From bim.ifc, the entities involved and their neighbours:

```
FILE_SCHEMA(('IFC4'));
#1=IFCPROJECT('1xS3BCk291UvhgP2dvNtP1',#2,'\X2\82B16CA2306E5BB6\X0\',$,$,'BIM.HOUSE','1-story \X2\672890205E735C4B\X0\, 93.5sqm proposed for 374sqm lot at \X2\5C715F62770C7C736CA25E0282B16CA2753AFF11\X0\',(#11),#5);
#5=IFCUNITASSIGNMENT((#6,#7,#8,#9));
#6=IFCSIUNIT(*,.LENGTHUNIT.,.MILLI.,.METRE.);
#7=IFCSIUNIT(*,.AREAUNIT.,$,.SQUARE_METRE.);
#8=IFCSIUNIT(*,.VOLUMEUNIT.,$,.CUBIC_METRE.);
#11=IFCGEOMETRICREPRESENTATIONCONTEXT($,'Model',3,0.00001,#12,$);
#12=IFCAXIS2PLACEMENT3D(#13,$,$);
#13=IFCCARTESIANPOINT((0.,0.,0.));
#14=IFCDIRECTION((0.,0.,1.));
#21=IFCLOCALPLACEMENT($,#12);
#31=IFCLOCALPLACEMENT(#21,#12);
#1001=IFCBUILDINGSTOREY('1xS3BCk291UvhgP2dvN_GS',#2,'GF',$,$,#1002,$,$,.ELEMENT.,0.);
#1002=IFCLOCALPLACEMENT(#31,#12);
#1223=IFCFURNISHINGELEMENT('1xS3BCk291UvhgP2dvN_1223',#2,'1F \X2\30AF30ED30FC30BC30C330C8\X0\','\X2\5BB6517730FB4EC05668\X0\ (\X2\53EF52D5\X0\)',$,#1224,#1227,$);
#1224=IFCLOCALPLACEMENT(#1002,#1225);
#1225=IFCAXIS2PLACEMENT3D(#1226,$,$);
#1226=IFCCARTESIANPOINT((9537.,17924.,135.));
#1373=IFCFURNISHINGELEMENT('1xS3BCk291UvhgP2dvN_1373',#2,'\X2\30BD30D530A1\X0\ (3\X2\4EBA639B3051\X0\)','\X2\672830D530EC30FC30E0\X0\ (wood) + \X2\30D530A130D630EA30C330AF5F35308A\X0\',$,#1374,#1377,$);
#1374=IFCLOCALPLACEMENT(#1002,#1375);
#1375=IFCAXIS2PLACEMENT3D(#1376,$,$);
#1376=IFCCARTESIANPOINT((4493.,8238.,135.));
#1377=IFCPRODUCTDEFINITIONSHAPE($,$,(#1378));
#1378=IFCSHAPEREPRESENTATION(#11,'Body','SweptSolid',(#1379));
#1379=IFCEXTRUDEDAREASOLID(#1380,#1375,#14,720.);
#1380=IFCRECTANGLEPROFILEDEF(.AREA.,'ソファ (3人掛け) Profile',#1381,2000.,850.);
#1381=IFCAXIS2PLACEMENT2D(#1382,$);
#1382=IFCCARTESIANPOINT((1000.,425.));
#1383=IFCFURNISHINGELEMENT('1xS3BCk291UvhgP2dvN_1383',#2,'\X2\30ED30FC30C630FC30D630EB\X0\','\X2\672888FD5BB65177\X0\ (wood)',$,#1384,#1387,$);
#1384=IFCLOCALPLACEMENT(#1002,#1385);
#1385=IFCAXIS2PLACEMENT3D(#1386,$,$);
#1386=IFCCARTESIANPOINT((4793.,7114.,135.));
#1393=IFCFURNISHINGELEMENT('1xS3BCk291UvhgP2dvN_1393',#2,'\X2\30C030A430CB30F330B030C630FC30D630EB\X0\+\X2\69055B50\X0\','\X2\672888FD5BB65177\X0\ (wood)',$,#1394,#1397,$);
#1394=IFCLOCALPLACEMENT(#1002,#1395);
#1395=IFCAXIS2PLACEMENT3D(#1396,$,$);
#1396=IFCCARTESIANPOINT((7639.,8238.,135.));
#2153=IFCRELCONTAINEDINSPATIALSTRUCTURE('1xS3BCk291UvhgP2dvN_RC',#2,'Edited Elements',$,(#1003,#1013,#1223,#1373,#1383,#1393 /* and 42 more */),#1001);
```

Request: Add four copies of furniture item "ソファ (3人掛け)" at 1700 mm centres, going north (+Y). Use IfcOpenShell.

```python
import numpy as np
import ifcopenshell
import ifcopenshell.api.geometry
import ifcopenshell.api.root
import ifcopenshell.util.element
import ifcopenshell.util.placement
import ifcopenshell.util.unit

model = ifcopenshell.open("bim.ifc")
unit_scale = ifcopenshell.util.unit.calculate_unit_scale(model)


def reuse_history(source, copy):
    """copy_class also copies each property set's owner history, people and application; keep the originals."""
    for rel in copy.IsDefinedBy:
        if rel.is_a("IfcRelDefinesByProperties") and (history := rel.RelatingPropertyDefinition.OwnerHistory):
            rel.RelatingPropertyDefinition.OwnerHistory = source.OwnerHistory
            ifcopenshell.util.element.remove_deep2(model, history)


source = model.by_guid("1xS3BCk291UvhgP2dvN_1373")
base = ifcopenshell.util.placement.get_local_placement(source.ObjectPlacement)
step = np.array([0.0, 1.0, 0.0]) * 1.7 / unit_scale

for i in range(1, 5):
    copy = ifcopenshell.api.root.copy_class(model, product=source)
    copy.Representation = ifcopenshell.util.element.copy_deep(
        model, source.Representation, exclude=["IfcGeometricRepresentationContext", "IfcRepresentationMap"]
    )
    reuse_history(source, copy)
    matrix = base.copy()
    matrix[:3, 3] += i * step
    print("added at", matrix[:3, 3].round(3) + 0.0)
    ifcopenshell.api.geometry.edit_object_placement(model, product=copy, matrix=matrix, is_si=False)

model.write("bim_updated.ifc")
```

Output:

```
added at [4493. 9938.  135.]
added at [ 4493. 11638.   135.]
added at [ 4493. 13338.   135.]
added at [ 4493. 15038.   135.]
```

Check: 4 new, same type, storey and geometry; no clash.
